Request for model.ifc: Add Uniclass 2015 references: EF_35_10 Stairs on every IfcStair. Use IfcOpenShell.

First a look at what the model holds.

```python
import ifcopenshell

model = ifcopenshell.open("model.ifc")
print(model.schema)
print("classifications:", [c.Name for c in model.by_type("IfcClassification")])
for ifc_class in ("IfcDoor", "IfcRoof", "IfcStair", "IfcWall", "IfcWindow"):
    print(ifc_class, len(model.by_type(ifc_class)))
```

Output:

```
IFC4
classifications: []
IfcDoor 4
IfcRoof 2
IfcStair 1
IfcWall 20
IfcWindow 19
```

```python
import ifcopenshell
import ifcopenshell.api.classification

model = ifcopenshell.open("model.ifc")

system = ifcopenshell.api.classification.add_classification(model, classification="Uniclass 2015")

codes = {
    "IfcStair": ("EF_35_10", "Stairs"),
}
for ifc_class, (code, name) in codes.items():
    products = model.by_type(ifc_class)
    ifcopenshell.api.classification.add_reference(
        model, products=products, classification=system, identification=code, name=name
    )
    print(code, len(products))

model.write("model_v2.ifc")
```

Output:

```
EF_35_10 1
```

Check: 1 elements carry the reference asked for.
